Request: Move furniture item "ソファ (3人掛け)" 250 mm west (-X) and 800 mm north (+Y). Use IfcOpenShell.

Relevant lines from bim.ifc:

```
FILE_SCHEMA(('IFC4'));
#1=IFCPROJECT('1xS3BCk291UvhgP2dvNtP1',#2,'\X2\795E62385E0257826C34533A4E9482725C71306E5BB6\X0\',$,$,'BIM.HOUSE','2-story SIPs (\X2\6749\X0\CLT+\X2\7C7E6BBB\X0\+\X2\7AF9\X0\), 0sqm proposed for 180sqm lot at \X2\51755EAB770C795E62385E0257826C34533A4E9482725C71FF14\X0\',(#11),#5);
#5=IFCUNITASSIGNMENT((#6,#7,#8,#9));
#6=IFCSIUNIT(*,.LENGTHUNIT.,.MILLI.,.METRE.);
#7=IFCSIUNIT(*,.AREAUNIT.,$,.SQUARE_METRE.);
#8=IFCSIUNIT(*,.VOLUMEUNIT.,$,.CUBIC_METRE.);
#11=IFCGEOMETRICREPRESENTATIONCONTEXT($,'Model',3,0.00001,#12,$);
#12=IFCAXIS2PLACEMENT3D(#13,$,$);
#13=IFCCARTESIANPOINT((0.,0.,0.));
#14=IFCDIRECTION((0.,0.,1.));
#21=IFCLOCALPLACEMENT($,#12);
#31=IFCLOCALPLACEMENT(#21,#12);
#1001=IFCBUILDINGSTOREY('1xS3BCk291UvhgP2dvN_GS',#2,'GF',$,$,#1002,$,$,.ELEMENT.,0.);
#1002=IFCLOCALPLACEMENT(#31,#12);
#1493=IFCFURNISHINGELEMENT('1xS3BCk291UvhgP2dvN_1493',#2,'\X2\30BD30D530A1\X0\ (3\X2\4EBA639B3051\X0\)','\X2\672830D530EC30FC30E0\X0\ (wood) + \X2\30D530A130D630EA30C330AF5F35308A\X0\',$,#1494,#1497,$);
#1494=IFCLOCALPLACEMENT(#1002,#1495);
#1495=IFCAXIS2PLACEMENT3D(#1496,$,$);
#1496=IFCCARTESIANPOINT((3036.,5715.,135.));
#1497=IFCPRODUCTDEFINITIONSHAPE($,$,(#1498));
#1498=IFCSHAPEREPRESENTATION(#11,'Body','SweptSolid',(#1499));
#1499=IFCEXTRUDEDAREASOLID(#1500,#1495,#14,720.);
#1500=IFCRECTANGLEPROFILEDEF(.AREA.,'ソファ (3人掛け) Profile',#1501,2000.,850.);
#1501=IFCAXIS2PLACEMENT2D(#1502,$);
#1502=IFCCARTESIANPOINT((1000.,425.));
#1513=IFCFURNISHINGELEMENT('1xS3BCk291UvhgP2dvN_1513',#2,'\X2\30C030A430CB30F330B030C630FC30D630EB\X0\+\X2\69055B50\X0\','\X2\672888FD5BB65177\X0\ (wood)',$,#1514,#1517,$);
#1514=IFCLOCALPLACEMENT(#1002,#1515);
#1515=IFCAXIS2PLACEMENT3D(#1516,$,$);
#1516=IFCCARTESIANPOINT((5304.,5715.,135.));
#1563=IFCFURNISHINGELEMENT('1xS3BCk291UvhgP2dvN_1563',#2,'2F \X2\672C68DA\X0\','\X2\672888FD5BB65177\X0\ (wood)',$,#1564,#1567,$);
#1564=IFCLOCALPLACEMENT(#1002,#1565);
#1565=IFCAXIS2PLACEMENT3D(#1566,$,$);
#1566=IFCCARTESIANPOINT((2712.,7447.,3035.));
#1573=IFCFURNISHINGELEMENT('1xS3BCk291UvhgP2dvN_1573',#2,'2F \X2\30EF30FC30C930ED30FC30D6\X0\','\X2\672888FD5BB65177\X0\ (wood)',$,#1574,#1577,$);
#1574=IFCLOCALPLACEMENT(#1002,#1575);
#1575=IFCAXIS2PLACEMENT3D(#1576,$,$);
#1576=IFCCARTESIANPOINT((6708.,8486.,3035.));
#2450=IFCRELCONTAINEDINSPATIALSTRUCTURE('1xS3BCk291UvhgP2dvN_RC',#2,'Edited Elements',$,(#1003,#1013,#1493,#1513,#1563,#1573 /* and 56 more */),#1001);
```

```python
import ifcopenshell
import ifcopenshell.api.geometry
import ifcopenshell.util.placement
import ifcopenshell.util.unit

model = ifcopenshell.open("bim.ifc")
unit_scale = ifcopenshell.util.unit.calculate_unit_scale(model)

item = model.by_guid("1xS3BCk291UvhgP2dvN_1493")
matrix = ifcopenshell.util.placement.get_local_placement(item.ObjectPlacement)
matrix[0, 3] -= 0.25 / unit_scale
matrix[1, 3] += 0.8 / unit_scale
ifcopenshell.api.geometry.edit_object_placement(model, product=item, matrix=matrix, is_si=False)

print(ifcopenshell.util.placement.get_local_placement(item.ObjectPlacement).round(3) + 0.0)

model.write("bim_updated.ifc")
```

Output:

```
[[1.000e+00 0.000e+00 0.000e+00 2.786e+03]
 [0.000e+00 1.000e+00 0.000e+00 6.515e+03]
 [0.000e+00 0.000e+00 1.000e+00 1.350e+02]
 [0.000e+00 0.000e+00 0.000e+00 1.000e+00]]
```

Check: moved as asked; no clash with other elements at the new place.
